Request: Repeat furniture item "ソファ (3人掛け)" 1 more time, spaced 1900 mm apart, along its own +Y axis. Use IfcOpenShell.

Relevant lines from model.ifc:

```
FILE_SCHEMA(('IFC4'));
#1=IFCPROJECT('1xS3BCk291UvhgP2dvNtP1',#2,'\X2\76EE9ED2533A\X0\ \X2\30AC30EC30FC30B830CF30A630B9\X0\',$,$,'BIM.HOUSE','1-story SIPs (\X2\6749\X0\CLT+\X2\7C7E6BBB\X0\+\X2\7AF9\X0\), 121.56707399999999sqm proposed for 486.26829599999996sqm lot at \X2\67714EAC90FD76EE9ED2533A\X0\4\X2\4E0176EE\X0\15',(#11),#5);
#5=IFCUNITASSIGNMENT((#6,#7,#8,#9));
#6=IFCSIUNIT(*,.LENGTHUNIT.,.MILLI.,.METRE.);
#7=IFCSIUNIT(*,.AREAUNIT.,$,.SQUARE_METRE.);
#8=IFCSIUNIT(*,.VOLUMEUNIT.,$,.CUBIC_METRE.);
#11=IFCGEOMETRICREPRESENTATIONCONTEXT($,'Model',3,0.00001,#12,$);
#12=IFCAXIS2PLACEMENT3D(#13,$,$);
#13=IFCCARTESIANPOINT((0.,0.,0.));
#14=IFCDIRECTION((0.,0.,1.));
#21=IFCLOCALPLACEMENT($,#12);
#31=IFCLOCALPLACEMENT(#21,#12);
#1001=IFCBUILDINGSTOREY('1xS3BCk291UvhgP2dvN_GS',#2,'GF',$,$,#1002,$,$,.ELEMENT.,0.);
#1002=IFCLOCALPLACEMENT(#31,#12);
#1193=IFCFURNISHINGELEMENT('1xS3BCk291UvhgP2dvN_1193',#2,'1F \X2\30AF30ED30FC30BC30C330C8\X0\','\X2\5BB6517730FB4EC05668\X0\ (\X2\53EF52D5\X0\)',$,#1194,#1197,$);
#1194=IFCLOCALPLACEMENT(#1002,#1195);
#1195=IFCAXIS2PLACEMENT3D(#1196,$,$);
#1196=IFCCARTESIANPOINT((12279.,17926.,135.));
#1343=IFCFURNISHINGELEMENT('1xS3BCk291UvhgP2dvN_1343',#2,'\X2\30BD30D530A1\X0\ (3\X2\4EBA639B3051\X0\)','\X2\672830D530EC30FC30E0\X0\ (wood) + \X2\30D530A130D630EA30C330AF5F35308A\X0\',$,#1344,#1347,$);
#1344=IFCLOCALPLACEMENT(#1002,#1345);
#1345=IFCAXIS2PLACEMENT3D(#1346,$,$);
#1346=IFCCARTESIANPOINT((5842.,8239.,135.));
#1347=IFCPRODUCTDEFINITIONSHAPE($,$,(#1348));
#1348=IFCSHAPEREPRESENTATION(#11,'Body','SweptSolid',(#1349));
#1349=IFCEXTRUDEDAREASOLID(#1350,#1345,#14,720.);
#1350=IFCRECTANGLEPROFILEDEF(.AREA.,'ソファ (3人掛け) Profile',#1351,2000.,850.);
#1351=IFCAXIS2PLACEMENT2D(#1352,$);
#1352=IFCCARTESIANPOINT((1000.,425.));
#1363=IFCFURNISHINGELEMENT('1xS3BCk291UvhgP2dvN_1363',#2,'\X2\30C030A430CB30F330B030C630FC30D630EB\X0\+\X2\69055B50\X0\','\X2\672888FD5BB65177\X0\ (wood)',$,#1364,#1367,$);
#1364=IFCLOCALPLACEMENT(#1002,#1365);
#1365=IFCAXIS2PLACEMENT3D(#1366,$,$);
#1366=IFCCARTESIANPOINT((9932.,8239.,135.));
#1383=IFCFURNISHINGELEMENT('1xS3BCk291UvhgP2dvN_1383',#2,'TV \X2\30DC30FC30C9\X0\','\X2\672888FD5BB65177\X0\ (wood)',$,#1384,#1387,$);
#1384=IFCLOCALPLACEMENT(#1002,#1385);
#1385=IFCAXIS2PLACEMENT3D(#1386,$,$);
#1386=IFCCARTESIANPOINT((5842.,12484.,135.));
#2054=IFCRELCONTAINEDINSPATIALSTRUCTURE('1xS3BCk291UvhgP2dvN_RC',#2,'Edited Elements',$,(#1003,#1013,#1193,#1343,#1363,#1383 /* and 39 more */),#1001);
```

```python
import ifcopenshell
import ifcopenshell.api.geometry
import ifcopenshell.api.root
import ifcopenshell.util.element
import ifcopenshell.util.placement
import ifcopenshell.util.unit

model = ifcopenshell.open("model.ifc")
unit_scale = ifcopenshell.util.unit.calculate_unit_scale(model)


def reuse_history(source, copy):
    """copy_class also copies each property set's owner history, people and application; keep the originals."""
    for rel in copy.IsDefinedBy:
        if rel.is_a("IfcRelDefinesByProperties") and (history := rel.RelatingPropertyDefinition.OwnerHistory):
            rel.RelatingPropertyDefinition.OwnerHistory = source.OwnerHistory
            ifcopenshell.util.element.remove_deep2(model, history)


source = model.by_guid("1xS3BCk291UvhgP2dvN_1343")
base = ifcopenshell.util.placement.get_local_placement(source.ObjectPlacement)
step = base[:3, 1] * 1.9 / unit_scale

for i in range(1, 2):
    copy = ifcopenshell.api.root.copy_class(model, product=source)
    copy.Representation = ifcopenshell.util.element.copy_deep(
        model, source.Representation, exclude=["IfcGeometricRepresentationContext", "IfcRepresentationMap"]
    )
    reuse_history(source, copy)
    matrix = base.copy()
    matrix[:3, 3] += i * step
    print("added at", matrix[:3, 3].round(3) + 0.0)
    ifcopenshell.api.geometry.edit_object_placement(model, product=copy, matrix=matrix, is_si=False)

model.write("model_v2.ifc")
```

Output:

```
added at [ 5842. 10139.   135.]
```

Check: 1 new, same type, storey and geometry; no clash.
